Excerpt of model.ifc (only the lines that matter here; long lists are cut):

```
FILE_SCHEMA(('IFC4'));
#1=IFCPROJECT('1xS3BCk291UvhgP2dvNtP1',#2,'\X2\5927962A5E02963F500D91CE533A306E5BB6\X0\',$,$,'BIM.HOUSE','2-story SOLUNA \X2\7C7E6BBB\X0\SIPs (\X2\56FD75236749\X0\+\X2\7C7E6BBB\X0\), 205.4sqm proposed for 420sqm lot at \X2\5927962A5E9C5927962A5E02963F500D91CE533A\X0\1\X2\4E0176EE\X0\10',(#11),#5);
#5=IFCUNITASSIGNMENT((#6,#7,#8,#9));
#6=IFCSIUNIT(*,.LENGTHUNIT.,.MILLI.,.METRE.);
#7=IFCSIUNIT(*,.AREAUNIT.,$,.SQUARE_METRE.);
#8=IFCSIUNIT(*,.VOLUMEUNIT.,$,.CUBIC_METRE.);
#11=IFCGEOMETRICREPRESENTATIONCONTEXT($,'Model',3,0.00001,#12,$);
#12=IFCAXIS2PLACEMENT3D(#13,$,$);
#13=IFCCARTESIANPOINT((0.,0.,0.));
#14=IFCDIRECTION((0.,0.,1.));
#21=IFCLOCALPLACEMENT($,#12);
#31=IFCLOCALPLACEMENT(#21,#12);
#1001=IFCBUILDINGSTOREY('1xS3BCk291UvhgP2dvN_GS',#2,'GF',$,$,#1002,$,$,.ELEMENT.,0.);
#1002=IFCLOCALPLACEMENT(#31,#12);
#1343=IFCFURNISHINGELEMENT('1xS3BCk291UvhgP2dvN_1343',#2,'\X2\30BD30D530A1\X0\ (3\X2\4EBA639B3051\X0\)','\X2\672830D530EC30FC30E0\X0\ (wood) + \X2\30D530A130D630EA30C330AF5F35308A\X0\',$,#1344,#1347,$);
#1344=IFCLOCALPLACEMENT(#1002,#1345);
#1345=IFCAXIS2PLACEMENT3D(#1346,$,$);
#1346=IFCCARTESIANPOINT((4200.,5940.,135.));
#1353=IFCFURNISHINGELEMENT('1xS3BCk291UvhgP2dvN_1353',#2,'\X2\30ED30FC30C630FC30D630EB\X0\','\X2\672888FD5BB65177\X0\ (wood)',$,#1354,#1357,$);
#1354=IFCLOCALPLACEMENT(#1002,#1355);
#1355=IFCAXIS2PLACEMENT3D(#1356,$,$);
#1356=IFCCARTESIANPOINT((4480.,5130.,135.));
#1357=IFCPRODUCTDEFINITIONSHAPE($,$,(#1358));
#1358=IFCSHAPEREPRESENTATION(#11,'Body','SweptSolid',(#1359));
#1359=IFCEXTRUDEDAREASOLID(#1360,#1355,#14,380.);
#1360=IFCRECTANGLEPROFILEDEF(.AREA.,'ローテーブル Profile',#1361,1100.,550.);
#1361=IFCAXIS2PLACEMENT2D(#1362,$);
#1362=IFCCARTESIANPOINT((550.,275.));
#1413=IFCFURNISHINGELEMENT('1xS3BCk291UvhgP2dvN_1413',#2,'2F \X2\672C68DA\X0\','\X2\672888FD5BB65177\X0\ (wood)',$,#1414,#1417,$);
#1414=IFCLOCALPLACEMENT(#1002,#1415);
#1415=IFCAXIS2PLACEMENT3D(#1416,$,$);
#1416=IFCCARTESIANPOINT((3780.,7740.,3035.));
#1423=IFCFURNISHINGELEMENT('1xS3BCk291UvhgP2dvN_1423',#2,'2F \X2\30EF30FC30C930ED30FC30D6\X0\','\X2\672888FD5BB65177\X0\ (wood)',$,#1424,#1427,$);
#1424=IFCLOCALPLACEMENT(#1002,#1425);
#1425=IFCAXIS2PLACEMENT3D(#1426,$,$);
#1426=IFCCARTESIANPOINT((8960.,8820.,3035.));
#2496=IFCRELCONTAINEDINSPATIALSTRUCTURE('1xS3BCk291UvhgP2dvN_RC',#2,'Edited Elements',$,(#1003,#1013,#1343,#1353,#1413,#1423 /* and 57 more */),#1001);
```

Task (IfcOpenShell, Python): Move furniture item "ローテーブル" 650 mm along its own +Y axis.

```python
import ifcopenshell
import ifcopenshell.api.geometry
import ifcopenshell.util.placement

model = ifcopenshell.open("model.ifc")

item = model.by_guid("1xS3BCk291UvhgP2dvN_1353")
matrix = ifcopenshell.util.placement.get_local_placement(item.ObjectPlacement)
matrix[:3, 3] += matrix[:3, 1] * 650.0
ifcopenshell.api.geometry.edit_object_placement(model, product=item, matrix=matrix, is_si=False)

print(ifcopenshell.util.placement.get_local_placement(item.ObjectPlacement).round(3) + 0.0)

model.write("model_updated.ifc")
```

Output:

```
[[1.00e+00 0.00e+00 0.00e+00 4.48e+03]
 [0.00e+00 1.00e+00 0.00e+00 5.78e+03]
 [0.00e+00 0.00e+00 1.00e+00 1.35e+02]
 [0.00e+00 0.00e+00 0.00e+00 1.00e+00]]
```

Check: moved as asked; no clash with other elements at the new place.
